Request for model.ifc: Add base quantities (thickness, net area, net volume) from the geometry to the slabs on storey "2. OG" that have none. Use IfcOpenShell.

First a look at what the model holds.

```python
import ifcopenshell
import ifcopenshell.util.element
import ifcopenshell.util.unit

model = ifcopenshell.open("model.ifc")
print(model.schema)
for unit_type in ("LENGTHUNIT", "AREAUNIT", "VOLUMEUNIT"):
    print(unit_type, ifcopenshell.util.unit.calculate_unit_scale(model, unit_type))
storey = next(s for s in model.by_type("IfcBuildingStorey") if s.Name == "2. OG")
slabs = [e for e in ifcopenshell.util.element.get_decomposition(storey) if e.is_a("IfcSlab")]
for e in sorted(slabs, key=lambda e: e.id()):
    print(e.id(), e.is_a(), e.Name, list(ifcopenshell.util.element.get_psets(e, qtos_only=True)), sep=" | ")
```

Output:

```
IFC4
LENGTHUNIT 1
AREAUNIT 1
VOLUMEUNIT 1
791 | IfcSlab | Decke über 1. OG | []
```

```python
import ifcopenshell
import ifcopenshell.api.pset
import ifcopenshell.geom
import ifcopenshell.util.element
import ifcopenshell.util.shape
import ifcopenshell.util.unit

model = ifcopenshell.open("model.ifc")
unit_scale = ifcopenshell.util.unit.calculate_unit_scale(model)
area_scale = ifcopenshell.util.unit.calculate_unit_scale(model, "AREAUNIT")
volume_scale = ifcopenshell.util.unit.calculate_unit_scale(model, "VOLUMEUNIT")
settings = ifcopenshell.geom.settings()

storey = next(s for s in model.by_type("IfcBuildingStorey") if s.Name == "2. OG")
slabs = [e for e in ifcopenshell.util.element.get_decomposition(storey) if e.is_a("IfcSlab")]

for e in sorted(slabs, key=lambda e: e.id()):
    if ifcopenshell.util.element.get_psets(e, qtos_only=True, should_inherit=False):
        continue
    # Geometry comes back in metres, in the element's own axes.
    shape = ifcopenshell.geom.create_shape(settings, e)
    values = {
        "Width": ifcopenshell.util.shape.get_z(shape.geometry) / unit_scale,
        "NetArea": ifcopenshell.util.shape.get_footprint_area(shape.geometry) / area_scale,
        "NetVolume": ifcopenshell.util.shape.get_volume(shape.geometry) / volume_scale,
    }
    qto = ifcopenshell.api.pset.add_qto(model, product=e, name="Qto_SlabBaseQuantities")
    ifcopenshell.api.pset.edit_qto(model, qto=qto, properties=values)
    print(e.id(), {k: round(v, 3) for k, v in values.items()})

model.write("model-out.ifc")
```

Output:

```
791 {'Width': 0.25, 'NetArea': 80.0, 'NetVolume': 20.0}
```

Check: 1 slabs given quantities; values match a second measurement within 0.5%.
